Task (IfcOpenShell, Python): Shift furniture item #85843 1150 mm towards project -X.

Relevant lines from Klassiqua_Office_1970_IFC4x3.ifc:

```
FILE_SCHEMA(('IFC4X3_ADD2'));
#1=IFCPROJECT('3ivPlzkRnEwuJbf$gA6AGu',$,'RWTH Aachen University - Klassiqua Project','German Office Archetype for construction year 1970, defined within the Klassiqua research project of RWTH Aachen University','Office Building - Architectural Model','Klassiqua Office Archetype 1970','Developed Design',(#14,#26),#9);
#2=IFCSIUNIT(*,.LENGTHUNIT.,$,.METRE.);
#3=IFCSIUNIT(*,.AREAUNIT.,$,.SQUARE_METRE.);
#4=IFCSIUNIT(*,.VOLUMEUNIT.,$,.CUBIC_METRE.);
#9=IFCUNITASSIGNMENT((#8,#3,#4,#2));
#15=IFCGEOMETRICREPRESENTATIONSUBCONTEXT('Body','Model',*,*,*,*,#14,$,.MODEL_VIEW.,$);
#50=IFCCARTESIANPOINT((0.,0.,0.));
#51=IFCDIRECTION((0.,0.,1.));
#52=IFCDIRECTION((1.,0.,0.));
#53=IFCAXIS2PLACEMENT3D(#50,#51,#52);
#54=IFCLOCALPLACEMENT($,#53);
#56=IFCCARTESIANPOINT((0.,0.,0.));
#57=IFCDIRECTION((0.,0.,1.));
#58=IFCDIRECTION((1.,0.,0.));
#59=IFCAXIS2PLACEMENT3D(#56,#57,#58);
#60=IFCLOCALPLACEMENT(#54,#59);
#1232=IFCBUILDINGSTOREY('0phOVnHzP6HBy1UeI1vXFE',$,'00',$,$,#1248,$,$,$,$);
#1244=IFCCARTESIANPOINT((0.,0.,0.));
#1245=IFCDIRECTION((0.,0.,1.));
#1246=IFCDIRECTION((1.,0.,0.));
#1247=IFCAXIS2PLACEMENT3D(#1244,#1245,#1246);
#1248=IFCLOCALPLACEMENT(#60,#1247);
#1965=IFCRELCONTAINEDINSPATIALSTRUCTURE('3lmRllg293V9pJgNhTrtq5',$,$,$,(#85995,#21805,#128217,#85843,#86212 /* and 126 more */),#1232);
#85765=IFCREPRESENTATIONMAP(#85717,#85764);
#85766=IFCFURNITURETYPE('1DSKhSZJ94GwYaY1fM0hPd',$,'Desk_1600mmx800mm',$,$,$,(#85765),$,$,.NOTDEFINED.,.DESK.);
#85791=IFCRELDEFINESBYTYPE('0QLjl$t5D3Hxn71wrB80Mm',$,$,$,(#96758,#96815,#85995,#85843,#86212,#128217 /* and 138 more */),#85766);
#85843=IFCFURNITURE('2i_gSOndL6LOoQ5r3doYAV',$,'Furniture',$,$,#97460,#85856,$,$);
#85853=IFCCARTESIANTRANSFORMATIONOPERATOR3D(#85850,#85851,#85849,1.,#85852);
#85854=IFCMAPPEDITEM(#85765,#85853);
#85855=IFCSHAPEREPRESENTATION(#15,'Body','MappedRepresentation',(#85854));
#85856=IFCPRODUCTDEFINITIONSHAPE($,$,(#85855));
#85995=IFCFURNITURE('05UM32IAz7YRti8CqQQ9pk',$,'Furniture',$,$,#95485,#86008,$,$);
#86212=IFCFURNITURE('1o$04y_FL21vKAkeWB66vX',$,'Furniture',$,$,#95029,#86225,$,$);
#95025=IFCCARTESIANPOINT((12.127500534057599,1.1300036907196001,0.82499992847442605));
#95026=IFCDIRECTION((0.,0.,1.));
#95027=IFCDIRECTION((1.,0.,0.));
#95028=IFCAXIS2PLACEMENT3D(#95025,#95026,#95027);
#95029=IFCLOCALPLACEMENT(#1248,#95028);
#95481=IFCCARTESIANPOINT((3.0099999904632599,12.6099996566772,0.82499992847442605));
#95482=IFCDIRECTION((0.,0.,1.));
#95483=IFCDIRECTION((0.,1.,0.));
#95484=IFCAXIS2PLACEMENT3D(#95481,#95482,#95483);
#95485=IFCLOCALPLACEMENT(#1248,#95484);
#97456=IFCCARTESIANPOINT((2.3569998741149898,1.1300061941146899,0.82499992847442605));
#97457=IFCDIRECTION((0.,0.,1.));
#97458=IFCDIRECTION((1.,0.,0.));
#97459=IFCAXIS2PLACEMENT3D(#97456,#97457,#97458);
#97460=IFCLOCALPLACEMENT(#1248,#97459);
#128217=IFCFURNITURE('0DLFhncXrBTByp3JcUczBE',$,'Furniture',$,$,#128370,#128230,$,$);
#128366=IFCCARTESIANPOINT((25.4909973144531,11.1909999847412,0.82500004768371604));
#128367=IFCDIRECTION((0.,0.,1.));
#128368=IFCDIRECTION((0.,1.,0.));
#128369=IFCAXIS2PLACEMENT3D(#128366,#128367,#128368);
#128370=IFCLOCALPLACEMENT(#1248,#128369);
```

```python
import ifcopenshell
import ifcopenshell.api.geometry
import ifcopenshell.util.placement

model = ifcopenshell.open("Klassiqua_Office_1970_IFC4x3.ifc")

item = model.by_guid("2i_gSOndL6LOoQ5r3doYAV")
matrix = ifcopenshell.util.placement.get_local_placement(item.ObjectPlacement)
matrix[0, 3] -= 1.15
ifcopenshell.api.geometry.edit_object_placement(model, product=item, matrix=matrix, is_si=False)

print(ifcopenshell.util.placement.get_local_placement(item.ObjectPlacement).round(3) + 0.0)

model.write("Klassiqua_Office_1970_IFC4x3_v2.ifc")
```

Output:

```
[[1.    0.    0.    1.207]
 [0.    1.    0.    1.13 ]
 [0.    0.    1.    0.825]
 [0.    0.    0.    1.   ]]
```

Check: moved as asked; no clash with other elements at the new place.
